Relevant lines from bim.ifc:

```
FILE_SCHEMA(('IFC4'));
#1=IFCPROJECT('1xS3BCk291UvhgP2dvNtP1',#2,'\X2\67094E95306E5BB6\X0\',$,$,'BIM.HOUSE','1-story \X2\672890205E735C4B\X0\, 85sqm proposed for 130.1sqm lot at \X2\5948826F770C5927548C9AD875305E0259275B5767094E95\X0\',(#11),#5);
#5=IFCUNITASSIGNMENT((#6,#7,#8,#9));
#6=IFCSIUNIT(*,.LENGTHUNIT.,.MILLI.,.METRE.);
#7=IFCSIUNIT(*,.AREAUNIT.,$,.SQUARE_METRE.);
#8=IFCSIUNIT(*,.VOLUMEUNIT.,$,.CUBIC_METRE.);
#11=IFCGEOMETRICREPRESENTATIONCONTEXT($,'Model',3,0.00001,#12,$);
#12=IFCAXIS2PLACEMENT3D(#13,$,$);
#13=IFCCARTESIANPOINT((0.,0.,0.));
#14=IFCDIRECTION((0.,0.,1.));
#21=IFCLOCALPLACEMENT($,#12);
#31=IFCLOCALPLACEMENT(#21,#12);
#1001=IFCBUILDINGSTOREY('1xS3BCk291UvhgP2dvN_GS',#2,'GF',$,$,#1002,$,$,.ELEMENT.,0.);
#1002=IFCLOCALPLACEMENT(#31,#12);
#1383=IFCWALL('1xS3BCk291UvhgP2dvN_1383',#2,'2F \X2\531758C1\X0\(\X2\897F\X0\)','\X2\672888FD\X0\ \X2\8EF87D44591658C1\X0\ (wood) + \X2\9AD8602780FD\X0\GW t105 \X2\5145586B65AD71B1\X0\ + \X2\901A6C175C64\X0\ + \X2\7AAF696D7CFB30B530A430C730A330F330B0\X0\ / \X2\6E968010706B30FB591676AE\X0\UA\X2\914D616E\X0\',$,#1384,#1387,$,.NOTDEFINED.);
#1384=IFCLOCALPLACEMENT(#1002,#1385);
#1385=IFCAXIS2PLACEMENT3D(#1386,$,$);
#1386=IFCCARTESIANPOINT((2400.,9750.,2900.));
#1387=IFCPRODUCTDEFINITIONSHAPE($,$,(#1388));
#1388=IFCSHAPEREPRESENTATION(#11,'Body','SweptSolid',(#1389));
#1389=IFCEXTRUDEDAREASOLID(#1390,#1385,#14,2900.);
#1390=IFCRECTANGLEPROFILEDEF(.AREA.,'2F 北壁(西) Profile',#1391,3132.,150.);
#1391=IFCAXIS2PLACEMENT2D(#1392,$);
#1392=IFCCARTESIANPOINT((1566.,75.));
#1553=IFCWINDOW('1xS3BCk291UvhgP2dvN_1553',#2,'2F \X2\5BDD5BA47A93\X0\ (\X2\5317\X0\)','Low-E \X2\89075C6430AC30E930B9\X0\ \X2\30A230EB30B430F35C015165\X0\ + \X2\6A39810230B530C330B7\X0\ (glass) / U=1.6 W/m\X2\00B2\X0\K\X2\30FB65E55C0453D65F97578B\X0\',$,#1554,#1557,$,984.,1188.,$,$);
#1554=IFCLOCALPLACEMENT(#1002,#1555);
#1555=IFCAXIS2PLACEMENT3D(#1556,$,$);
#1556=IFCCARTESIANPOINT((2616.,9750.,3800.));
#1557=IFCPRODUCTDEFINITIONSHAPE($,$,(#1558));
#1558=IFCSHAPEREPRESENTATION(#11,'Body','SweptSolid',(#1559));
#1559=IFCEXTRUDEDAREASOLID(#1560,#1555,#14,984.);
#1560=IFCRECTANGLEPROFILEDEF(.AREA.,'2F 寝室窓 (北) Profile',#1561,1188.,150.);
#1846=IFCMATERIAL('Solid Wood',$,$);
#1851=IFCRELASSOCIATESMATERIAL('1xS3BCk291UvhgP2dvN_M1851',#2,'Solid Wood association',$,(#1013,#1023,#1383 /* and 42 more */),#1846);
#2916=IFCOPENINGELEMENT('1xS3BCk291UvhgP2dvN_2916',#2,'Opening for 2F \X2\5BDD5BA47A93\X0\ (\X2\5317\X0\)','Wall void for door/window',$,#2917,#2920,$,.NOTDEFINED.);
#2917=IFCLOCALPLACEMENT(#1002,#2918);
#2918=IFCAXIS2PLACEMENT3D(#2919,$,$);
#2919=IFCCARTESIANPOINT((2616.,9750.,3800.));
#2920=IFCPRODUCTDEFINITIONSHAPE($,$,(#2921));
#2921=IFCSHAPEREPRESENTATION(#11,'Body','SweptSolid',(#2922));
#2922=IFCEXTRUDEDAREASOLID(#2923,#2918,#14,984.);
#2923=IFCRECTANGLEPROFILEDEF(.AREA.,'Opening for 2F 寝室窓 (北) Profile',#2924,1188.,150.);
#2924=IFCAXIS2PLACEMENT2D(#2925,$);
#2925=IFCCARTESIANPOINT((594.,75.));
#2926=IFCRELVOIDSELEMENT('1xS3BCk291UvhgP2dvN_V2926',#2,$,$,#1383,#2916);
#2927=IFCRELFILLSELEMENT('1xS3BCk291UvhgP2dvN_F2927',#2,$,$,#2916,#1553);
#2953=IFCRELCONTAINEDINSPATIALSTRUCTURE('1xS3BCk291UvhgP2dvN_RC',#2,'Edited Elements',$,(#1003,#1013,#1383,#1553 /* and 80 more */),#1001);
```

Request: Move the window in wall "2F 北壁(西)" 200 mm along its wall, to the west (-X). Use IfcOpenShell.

```python
import ifcopenshell
import ifcopenshell.api.geometry
import ifcopenshell.util.placement
import ifcopenshell.util.unit

model = ifcopenshell.open("bim.ifc")
unit_scale = ifcopenshell.util.unit.calculate_unit_scale(model)

window = model.by_id(1553)
opening = window.FillsVoids[0].RelatingOpeningElement
wall = opening.VoidsElements[0].RelatingBuildingElement

wall_matrix = ifcopenshell.util.placement.get_local_placement(wall.ObjectPlacement)
shift = wall_matrix[:3, 0] * -0.2 / unit_scale
before = ifcopenshell.util.placement.get_local_placement(window.ObjectPlacement)[:3, 3].copy()

# The window is not placed relative to its opening, so move both.
for product in (opening, window):
    matrix = ifcopenshell.util.placement.get_local_placement(product.ObjectPlacement)
    matrix[:3, 3] += shift
    ifcopenshell.api.geometry.edit_object_placement(model, product=product, matrix=matrix, is_si=False)

after = ifcopenshell.util.placement.get_local_placement(window.ObjectPlacement)[:3, 3]
print("window moved by", (after - before).round(3) + 0.0)

model.write("bim-out.ifc")
```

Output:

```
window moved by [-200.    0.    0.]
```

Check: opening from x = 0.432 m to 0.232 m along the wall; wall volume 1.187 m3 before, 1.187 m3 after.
